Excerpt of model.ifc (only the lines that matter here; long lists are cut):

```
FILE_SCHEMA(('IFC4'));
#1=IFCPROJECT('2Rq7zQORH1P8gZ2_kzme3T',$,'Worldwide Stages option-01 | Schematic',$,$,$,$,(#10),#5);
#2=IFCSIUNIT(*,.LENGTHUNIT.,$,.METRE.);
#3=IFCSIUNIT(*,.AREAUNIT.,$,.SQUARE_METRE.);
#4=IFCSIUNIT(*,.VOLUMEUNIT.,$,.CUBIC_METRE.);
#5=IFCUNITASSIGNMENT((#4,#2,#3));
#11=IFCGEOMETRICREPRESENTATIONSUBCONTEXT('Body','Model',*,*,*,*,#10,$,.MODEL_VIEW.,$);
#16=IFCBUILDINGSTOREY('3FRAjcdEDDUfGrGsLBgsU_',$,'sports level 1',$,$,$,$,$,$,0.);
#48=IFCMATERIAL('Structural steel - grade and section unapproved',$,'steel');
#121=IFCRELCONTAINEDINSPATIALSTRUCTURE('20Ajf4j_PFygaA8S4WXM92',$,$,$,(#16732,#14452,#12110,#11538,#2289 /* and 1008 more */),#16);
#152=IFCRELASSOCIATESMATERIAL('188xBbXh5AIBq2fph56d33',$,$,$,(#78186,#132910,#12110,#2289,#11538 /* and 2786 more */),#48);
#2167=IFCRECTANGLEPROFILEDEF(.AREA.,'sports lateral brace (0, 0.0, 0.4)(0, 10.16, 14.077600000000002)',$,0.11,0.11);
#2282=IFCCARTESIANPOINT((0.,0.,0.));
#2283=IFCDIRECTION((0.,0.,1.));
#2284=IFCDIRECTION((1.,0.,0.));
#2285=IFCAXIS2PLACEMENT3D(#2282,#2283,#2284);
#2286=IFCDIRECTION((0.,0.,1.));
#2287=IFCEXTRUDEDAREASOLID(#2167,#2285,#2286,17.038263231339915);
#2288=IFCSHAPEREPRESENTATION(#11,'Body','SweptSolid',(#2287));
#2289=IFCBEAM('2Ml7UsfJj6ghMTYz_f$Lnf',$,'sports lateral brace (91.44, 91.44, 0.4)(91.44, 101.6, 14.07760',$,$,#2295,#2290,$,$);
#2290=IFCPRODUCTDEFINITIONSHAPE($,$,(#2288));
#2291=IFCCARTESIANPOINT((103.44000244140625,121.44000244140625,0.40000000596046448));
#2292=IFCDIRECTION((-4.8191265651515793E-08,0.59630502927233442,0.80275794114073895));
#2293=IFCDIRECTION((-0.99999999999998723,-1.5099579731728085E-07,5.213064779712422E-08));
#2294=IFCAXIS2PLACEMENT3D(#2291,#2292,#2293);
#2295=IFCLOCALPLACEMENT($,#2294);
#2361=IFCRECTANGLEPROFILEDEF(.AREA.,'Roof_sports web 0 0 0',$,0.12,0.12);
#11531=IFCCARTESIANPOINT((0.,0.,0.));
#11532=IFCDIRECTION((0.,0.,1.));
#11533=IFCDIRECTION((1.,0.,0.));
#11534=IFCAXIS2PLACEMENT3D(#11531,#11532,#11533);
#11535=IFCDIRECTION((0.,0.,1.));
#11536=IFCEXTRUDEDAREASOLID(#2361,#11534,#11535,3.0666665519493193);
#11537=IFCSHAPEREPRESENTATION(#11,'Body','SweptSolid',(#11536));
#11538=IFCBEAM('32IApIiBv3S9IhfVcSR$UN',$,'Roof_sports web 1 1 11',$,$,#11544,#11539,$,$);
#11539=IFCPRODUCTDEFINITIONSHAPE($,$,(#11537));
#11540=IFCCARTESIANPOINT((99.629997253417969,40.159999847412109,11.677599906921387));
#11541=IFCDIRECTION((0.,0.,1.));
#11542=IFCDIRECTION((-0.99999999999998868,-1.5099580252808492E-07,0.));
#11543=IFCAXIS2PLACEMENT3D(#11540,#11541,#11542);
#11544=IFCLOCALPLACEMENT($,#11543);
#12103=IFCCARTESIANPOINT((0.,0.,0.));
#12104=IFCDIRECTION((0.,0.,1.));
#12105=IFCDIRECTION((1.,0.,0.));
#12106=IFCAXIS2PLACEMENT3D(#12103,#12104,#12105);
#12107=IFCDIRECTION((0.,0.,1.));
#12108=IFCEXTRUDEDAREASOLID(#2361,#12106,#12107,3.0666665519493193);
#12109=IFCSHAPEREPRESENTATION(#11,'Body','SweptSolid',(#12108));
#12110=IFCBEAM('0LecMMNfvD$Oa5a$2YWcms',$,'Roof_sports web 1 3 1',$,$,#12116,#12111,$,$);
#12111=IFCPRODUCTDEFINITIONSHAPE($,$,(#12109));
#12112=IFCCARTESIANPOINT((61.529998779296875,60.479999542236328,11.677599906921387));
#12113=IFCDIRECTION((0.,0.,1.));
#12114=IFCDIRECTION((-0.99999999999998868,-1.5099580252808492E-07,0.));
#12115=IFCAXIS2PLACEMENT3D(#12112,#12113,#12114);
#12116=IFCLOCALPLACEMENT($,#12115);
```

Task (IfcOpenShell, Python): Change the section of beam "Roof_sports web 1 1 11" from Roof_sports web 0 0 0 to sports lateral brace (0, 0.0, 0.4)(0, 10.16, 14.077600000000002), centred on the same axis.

```python
import ifcopenshell
import ifcopenshell.util.element
import ifcopenshell.util.representation

model = ifcopenshell.open("model.ifc")

member = model.by_guid("32IApIiBv3S9IhfVcSR$UN")
source = next(p for p in model.by_type("IfcRectangleProfileDef") if p.ProfileName == "sports lateral brace (0, 0.0, 0.4)(0, 10.16, 14.077600000000002)")

body = ifcopenshell.util.representation.get_representation(member, "Model", "Body")
solid = body.Items[0]
old_profile = solid.SweptArea

# Copy the section's sizes but keep this member's own profile position.
profile = ifcopenshell.util.element.copy(model, source)
profile.Position = old_profile.Position
solid.SweptArea = profile
if not model.get_total_inverses(old_profile):
    ifcopenshell.util.element.remove_deep2(model, old_profile)

print(solid.SweptArea)

model.write("model_v2.ifc")
```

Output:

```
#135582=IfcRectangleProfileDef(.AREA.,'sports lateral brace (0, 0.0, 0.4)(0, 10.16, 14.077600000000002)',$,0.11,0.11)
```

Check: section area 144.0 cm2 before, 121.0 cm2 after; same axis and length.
